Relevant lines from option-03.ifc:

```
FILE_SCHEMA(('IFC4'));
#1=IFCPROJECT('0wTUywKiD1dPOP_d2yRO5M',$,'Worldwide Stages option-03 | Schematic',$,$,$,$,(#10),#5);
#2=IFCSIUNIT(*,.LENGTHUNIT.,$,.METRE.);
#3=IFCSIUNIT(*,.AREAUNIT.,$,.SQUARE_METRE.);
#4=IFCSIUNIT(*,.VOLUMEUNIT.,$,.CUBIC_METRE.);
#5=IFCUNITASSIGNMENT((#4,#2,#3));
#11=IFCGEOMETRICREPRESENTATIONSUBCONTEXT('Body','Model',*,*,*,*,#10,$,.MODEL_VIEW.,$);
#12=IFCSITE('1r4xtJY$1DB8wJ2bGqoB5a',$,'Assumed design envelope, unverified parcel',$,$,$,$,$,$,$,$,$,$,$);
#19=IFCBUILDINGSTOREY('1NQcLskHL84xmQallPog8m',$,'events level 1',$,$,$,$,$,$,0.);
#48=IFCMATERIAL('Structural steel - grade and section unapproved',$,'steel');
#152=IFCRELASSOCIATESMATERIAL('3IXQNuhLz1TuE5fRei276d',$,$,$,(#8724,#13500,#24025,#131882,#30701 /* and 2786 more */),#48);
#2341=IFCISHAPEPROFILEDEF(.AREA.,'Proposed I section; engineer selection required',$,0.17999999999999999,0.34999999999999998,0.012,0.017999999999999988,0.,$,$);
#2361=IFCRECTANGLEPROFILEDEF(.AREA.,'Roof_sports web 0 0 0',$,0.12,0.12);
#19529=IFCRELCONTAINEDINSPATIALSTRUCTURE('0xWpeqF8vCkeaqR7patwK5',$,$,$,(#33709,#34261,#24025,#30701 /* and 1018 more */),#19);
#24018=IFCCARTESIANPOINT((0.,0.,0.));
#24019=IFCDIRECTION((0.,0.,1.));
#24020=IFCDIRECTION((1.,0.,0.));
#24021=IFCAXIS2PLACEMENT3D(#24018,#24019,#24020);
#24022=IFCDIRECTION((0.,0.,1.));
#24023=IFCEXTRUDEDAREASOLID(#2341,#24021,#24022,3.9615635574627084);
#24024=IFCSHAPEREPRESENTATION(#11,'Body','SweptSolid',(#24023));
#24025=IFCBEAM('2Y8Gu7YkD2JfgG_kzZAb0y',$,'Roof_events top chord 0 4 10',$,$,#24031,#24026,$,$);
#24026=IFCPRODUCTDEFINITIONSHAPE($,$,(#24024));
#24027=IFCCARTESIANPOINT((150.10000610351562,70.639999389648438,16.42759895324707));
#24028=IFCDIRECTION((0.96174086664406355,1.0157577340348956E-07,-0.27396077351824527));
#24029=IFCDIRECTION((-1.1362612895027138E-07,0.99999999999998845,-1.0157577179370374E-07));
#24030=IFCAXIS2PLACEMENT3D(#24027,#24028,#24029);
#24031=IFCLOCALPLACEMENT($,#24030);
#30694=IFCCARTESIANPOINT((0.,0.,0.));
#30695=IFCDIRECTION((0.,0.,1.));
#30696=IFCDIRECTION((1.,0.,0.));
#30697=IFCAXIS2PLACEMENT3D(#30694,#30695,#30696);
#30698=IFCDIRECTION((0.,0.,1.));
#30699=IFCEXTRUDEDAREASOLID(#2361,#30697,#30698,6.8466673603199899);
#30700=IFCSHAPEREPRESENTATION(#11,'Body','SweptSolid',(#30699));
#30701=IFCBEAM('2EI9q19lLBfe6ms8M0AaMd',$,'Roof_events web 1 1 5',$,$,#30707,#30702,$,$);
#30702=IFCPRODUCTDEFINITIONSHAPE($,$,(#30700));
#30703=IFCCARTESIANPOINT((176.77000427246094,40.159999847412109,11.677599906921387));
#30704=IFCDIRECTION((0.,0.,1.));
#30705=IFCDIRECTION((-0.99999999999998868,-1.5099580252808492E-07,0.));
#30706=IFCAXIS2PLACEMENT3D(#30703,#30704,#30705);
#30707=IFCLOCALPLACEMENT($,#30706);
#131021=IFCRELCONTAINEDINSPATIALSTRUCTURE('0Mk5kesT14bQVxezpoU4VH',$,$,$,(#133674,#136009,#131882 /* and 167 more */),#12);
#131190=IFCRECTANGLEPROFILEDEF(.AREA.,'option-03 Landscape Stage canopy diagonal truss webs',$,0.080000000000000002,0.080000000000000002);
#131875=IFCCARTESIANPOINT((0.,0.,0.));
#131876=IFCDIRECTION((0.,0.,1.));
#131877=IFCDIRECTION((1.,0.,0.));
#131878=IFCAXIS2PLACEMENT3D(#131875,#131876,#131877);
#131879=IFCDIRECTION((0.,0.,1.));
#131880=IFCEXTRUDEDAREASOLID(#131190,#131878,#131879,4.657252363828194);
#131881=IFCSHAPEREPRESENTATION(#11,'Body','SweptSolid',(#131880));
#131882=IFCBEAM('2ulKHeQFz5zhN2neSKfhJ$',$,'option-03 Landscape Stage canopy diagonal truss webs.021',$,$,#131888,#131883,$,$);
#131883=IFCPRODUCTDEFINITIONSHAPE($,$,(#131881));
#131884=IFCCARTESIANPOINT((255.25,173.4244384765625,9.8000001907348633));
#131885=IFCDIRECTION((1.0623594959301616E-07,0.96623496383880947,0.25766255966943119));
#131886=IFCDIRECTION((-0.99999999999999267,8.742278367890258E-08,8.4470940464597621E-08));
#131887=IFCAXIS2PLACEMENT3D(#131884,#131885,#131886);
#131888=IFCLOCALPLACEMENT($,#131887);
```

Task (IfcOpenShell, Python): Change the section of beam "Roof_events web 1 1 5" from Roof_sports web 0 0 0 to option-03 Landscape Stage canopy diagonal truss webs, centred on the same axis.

```python
import ifcopenshell
import ifcopenshell.util.element
import ifcopenshell.util.representation

model = ifcopenshell.open("option-03.ifc")

member = model.by_guid("2EI9q19lLBfe6ms8M0AaMd")
source = next(p for p in model.by_type("IfcRectangleProfileDef") if p.ProfileName == "option-03 Landscape Stage canopy diagonal truss webs")

body = ifcopenshell.util.representation.get_representation(member, "Model", "Body")
solid = body.Items[0]
old_profile = solid.SweptArea

# Copy the section's sizes but keep this member's own profile position.
profile = ifcopenshell.util.element.copy(model, source)
profile.Position = old_profile.Position
solid.SweptArea = profile
if not model.get_total_inverses(old_profile):
    ifcopenshell.util.element.remove_deep2(model, old_profile)

print(solid.SweptArea)

model.write("option-03_rev.ifc")
```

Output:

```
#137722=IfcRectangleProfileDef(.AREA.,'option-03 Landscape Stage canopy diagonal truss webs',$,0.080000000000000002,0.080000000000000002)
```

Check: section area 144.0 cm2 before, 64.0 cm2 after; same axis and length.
